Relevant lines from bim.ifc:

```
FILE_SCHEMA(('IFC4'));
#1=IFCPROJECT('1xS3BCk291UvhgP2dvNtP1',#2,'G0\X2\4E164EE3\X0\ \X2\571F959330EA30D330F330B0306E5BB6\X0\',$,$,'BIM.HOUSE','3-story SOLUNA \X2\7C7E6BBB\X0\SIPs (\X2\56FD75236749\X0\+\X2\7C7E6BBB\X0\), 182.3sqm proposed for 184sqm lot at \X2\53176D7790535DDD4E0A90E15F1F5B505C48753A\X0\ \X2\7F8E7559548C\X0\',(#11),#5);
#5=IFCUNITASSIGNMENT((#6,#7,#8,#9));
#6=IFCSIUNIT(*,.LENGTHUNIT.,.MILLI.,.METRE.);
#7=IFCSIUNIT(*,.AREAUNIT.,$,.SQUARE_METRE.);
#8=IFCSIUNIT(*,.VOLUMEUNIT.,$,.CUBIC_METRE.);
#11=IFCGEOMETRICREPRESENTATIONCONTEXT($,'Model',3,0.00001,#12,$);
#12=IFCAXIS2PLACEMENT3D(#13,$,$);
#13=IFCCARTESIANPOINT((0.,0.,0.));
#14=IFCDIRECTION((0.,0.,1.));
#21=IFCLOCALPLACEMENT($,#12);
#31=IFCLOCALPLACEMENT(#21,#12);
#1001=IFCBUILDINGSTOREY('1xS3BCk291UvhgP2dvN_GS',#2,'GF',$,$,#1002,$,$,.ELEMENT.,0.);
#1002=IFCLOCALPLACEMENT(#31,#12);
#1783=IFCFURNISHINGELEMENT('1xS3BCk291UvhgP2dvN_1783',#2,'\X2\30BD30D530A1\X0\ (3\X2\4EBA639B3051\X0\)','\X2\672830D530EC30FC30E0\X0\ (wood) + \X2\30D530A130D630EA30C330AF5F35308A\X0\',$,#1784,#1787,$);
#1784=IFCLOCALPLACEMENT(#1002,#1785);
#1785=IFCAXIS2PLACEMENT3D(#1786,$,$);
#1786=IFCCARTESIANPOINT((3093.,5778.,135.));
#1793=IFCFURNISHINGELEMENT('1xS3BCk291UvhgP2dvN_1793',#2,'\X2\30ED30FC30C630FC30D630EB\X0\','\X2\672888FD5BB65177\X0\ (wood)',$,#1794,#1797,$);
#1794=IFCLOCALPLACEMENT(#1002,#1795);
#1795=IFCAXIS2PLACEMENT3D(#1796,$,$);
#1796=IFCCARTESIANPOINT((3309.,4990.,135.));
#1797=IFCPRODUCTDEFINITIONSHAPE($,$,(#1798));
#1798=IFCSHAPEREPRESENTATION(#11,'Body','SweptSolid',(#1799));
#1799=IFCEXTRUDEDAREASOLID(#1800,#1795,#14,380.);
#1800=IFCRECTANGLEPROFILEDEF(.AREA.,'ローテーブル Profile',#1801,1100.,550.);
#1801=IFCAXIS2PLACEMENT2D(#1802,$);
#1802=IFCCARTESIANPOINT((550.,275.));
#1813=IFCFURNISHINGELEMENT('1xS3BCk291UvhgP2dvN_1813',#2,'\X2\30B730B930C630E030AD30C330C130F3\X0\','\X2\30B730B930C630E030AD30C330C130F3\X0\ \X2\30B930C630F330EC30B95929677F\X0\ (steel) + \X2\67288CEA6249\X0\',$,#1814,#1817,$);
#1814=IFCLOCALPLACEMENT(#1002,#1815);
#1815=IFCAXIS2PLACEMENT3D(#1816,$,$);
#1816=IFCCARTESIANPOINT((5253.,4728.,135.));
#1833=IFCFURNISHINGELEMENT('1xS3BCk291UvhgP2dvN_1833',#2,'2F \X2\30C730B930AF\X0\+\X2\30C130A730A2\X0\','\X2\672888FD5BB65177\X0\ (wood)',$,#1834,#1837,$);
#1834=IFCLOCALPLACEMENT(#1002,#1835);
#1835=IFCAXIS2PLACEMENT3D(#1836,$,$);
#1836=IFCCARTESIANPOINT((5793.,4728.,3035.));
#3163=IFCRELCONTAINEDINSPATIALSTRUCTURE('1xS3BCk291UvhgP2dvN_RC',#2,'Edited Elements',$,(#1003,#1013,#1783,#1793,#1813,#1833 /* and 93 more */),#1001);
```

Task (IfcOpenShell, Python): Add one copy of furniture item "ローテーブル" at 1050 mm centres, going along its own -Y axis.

```python
import ifcopenshell
import ifcopenshell.api.geometry
import ifcopenshell.api.root
import ifcopenshell.util.element
import ifcopenshell.util.placement

model = ifcopenshell.open("bim.ifc")


def reuse_history(source, copy):
    """copy_class also copies each property set's owner history, people and application; keep the originals."""
    for rel in copy.IsDefinedBy:
        if rel.is_a("IfcRelDefinesByProperties") and (history := rel.RelatingPropertyDefinition.OwnerHistory):
            rel.RelatingPropertyDefinition.OwnerHistory = source.OwnerHistory
            ifcopenshell.util.element.remove_deep2(model, history)


source = model.by_guid("1xS3BCk291UvhgP2dvN_1793")
base = ifcopenshell.util.placement.get_local_placement(source.ObjectPlacement)
step = -base[:3, 1] * 1050.0

for i in range(1, 2):
    copy = ifcopenshell.api.root.copy_class(model, product=source)
    copy.Representation = ifcopenshell.util.element.copy_deep(
        model, source.Representation, exclude=["IfcGeometricRepresentationContext", "IfcRepresentationMap"]
    )
    reuse_history(source, copy)
    matrix = base.copy()
    matrix[:3, 3] += i * step
    print("added at", matrix[:3, 3].round(3) + 0.0)
    ifcopenshell.api.geometry.edit_object_placement(model, product=copy, matrix=matrix, is_si=False)

model.write("bim-out.ifc")
```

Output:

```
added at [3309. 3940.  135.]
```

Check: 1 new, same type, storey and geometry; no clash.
